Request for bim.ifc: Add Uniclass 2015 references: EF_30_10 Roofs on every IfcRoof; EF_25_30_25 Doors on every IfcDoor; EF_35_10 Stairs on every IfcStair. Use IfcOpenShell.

First a look at what the model holds.

```python
import ifcopenshell

model = ifcopenshell.open("bim.ifc")
print(model.schema)
print("classifications:", [c.Name for c in model.by_type("IfcClassification")])
for ifc_class in ("IfcDoor", "IfcRoof", "IfcStair", "IfcWall", "IfcWindow"):
    print(ifc_class, len(model.by_type(ifc_class)))
```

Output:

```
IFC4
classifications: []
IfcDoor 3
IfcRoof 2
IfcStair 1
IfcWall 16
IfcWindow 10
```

```python
import ifcopenshell
import ifcopenshell.api.classification

model = ifcopenshell.open("bim.ifc")

system = ifcopenshell.api.classification.add_classification(model, classification="Uniclass 2015")

codes = {
    "IfcRoof": ("EF_30_10", "Roofs"),
    "IfcDoor": ("EF_25_30_25", "Doors"),
    "IfcStair": ("EF_35_10", "Stairs"),
}
for ifc_class, (code, name) in codes.items():
    products = model.by_type(ifc_class)
    ifcopenshell.api.classification.add_reference(
        model, products=products, classification=system, identification=code, name=name
    )
    print(code, len(products))

model.write("bim_v2.ifc")
```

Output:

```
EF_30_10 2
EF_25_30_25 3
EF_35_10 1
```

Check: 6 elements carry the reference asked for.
